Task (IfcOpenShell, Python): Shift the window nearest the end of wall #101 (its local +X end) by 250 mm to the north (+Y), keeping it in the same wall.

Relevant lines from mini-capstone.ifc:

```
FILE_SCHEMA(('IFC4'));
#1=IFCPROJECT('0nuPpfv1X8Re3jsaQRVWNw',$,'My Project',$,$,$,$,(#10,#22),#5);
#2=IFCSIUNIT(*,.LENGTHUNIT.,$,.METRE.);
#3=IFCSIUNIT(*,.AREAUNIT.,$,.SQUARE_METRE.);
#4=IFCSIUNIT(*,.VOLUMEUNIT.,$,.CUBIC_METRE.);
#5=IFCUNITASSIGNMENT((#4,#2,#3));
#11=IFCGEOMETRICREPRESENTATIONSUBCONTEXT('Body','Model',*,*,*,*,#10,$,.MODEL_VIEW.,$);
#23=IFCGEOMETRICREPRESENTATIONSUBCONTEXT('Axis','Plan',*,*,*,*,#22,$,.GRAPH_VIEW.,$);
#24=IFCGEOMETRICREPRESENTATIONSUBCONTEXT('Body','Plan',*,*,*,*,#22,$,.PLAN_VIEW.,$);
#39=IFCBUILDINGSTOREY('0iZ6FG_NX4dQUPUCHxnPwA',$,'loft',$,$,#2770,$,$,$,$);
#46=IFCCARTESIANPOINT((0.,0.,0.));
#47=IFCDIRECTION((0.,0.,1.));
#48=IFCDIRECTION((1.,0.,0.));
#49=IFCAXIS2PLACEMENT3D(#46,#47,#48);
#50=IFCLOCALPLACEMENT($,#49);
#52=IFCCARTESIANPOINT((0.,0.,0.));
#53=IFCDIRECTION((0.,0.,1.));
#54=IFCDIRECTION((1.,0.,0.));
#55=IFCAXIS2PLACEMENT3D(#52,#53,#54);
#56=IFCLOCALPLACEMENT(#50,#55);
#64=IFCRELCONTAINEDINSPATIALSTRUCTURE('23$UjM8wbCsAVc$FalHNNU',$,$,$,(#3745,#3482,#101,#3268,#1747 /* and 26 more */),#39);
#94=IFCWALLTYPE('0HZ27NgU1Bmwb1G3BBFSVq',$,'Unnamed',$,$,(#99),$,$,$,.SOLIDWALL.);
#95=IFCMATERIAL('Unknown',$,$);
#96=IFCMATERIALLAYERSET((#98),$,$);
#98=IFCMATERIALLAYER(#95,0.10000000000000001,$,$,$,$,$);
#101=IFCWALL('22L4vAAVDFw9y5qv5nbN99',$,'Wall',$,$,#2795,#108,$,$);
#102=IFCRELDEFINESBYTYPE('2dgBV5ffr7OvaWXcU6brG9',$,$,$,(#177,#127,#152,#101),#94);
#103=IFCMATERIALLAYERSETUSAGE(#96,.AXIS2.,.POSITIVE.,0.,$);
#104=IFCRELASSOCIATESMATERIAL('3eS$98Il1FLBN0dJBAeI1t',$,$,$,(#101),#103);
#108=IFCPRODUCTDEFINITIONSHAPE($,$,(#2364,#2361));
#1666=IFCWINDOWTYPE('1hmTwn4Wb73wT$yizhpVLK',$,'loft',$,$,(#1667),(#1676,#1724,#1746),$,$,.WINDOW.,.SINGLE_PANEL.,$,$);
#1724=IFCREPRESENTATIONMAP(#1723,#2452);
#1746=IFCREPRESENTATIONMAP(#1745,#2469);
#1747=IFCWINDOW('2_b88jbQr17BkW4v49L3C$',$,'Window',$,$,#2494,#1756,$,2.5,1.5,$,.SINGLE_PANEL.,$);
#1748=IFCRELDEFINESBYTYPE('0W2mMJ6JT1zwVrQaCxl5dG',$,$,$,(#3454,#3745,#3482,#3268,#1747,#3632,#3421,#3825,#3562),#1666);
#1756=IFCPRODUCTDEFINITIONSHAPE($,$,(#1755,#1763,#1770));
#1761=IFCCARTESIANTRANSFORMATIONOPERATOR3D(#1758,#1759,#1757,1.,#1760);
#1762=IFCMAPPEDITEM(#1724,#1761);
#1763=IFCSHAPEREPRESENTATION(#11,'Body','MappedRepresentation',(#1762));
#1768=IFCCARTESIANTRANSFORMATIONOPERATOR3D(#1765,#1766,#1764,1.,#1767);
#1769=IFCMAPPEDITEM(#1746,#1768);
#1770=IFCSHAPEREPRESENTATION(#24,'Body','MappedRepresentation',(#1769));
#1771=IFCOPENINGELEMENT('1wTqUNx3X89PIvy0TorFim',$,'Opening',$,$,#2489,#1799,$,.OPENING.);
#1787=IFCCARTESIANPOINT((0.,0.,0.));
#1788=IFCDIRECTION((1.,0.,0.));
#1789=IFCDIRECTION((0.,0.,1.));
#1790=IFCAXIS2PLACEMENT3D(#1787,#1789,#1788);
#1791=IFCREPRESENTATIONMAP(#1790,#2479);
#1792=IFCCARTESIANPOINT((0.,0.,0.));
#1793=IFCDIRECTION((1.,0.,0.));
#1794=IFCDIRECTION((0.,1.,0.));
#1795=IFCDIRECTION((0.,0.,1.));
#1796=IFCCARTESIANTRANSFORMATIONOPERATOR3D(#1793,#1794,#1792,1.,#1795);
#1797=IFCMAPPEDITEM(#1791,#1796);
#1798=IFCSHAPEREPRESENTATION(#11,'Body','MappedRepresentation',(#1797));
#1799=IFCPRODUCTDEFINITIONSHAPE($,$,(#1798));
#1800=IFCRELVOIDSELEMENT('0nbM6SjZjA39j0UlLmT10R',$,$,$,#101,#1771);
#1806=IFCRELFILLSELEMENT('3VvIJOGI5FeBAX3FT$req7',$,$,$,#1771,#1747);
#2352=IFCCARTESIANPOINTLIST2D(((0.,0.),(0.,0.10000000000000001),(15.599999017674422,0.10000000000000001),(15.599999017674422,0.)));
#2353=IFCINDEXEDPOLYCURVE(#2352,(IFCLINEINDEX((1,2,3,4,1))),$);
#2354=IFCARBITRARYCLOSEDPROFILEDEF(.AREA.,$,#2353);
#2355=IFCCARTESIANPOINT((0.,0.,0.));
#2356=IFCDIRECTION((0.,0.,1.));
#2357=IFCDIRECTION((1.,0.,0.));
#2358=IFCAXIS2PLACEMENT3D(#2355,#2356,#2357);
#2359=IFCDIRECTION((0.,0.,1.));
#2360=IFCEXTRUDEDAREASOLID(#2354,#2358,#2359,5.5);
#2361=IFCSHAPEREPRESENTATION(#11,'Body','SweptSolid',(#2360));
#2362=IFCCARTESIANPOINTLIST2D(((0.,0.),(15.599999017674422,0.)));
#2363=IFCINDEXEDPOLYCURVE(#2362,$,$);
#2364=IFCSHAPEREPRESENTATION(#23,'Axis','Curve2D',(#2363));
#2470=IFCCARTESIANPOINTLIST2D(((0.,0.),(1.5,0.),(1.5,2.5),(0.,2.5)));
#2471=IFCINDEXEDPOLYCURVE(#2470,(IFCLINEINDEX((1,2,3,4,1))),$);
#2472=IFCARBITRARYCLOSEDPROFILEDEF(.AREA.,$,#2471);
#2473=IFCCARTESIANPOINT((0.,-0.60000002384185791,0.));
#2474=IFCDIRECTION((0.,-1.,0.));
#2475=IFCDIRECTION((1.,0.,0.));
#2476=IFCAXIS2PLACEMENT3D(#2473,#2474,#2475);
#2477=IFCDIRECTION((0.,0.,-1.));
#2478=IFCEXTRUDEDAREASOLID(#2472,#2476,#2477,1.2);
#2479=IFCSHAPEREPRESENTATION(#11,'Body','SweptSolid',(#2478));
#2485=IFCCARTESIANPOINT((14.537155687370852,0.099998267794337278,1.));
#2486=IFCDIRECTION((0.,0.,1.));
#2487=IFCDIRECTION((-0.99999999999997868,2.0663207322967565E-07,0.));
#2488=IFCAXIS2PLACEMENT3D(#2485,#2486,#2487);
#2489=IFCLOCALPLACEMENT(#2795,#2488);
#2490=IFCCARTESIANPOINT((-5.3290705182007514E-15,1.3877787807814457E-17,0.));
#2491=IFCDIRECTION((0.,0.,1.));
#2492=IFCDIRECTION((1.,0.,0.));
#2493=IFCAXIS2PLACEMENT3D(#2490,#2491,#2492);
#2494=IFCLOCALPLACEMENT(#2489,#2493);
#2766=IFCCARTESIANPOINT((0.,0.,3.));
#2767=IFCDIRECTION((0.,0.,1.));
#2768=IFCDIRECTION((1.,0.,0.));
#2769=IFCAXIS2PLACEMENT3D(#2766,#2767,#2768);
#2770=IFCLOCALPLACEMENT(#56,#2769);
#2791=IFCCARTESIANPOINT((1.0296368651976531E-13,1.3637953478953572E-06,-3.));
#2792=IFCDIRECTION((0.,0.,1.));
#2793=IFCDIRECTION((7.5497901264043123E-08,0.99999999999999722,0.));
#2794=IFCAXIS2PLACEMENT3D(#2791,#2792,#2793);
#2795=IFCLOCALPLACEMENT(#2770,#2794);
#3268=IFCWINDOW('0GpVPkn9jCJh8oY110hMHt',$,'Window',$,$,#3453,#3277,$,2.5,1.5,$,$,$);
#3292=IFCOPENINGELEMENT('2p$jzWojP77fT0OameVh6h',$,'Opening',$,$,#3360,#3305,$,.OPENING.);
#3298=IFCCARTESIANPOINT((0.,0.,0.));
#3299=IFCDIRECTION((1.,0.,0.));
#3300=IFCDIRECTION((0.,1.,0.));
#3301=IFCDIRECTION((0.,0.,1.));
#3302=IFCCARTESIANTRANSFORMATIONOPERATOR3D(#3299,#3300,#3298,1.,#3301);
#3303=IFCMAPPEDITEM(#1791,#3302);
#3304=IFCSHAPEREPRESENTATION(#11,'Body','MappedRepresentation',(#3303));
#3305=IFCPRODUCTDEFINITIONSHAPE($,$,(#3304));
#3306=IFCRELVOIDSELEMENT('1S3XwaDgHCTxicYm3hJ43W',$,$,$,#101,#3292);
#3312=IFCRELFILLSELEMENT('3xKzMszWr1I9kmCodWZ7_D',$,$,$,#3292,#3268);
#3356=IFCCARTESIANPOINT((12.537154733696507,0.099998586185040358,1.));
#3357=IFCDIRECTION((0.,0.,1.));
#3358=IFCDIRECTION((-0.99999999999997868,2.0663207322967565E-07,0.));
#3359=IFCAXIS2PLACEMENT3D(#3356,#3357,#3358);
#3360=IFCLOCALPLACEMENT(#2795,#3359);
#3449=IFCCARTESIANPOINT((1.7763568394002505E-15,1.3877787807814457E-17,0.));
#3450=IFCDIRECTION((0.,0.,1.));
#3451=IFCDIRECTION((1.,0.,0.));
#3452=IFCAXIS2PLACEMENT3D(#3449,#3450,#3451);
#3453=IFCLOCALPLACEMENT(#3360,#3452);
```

```python
import ifcopenshell
import ifcopenshell.api.geometry
import ifcopenshell.util.placement
import ifcopenshell.util.unit

model = ifcopenshell.open("mini-capstone.ifc")
unit_scale = ifcopenshell.util.unit.calculate_unit_scale(model)

window = model.by_guid("2_b88jbQr17BkW4v49L3C$")
opening = window.FillsVoids[0].RelatingOpeningElement
wall = opening.VoidsElements[0].RelatingBuildingElement

wall_matrix = ifcopenshell.util.placement.get_local_placement(wall.ObjectPlacement)
shift = wall_matrix[:3, 0] * 0.25 / unit_scale
before = ifcopenshell.util.placement.get_local_placement(window.ObjectPlacement)[:3, 3].copy()

# The window is placed relative to its opening, so it follows when the opening moves.
matrix = ifcopenshell.util.placement.get_local_placement(opening.ObjectPlacement)
matrix[:3, 3] += shift
ifcopenshell.api.geometry.edit_object_placement(
    model, product=opening, matrix=matrix, is_si=False, should_transform_children=True
)

after = ifcopenshell.util.placement.get_local_placement(window.ObjectPlacement)[:3, 3]
print("window moved by", (after - before).round(3) + 0.0)

model.write("mini-capstone_rev.ifc")
```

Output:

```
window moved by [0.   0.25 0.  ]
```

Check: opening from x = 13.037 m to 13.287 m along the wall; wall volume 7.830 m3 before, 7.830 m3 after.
